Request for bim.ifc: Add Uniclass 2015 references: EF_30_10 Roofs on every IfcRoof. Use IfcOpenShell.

First a look at what the model holds.

```python
import ifcopenshell

model = ifcopenshell.open("bim.ifc")
print(model.schema)
print("classifications:", [c.Name for c in model.by_type("IfcClassification")])
for ifc_class in ("IfcDoor", "IfcRoof", "IfcStair", "IfcWall", "IfcWindow"):
    print(ifc_class, len(model.by_type(ifc_class)))
```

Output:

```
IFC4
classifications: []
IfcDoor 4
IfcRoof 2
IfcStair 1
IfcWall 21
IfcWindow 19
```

```python
import ifcopenshell
import ifcopenshell.api.classification

model = ifcopenshell.open("bim.ifc")

system = ifcopenshell.api.classification.add_classification(model, classification="Uniclass 2015")

codes = {
    "IfcRoof": ("EF_30_10", "Roofs"),
}
for ifc_class, (code, name) in codes.items():
    products = model.by_type(ifc_class)
    ifcopenshell.api.classification.add_reference(
        model, products=products, classification=system, identification=code, name=name
    )
    print(code, len(products))

model.write("bim_v2.ifc")
```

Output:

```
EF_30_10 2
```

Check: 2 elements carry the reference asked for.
